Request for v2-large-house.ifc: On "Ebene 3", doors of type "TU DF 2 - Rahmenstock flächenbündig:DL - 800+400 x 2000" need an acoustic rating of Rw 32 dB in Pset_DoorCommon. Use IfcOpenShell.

First a look at what the model holds.

```python
import ifcopenshell
import ifcopenshell.util.element

model = ifcopenshell.open("v2-large-house.ifc")
print(model.schema)
storey = next(s for s in model.by_type("IfcBuildingStorey") if s.Name == "Ebene 3")
doors = [e for e in ifcopenshell.util.element.get_decomposition(storey) if e.is_a("IfcDoor")]
seen = {}
for e in doors:
    element_type = ifcopenshell.util.element.get_type(e)
    key = (element_type.Name if element_type != e and element_type else None, ifcopenshell.util.element.get_pset(e, "Pset_DoorCommon", "AcousticRating"))
    seen[key] = seen.get(key, 0) + 1
for (name, value), count in sorted(seen.items(), key=str):
    print(count, "x", name, "|", value)
```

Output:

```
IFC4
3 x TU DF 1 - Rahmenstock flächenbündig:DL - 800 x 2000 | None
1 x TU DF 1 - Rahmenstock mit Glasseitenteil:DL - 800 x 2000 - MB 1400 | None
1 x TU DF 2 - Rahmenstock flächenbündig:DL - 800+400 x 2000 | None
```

```python
import ifcopenshell
import ifcopenshell.api.pset
import ifcopenshell.util.element

model = ifcopenshell.open("v2-large-house.ifc")

storey = next(s for s in model.by_type("IfcBuildingStorey") if s.Name == "Ebene 3")
doors = [e for e in ifcopenshell.util.element.get_decomposition(storey) if e.is_a("IfcDoor")]

count = 0
for e in doors:
    element_type = ifcopenshell.util.element.get_type(e)
    if element_type in (None, e) or element_type.Name != "TU DF 2 - Rahmenstock flächenbündig:DL - 800+400 x 2000":
        continue
    # add_pset returns the element's existing set when there is one.
    pset = ifcopenshell.api.pset.add_pset(model, product=e, name="Pset_DoorCommon")
    ifcopenshell.api.pset.edit_pset(model, pset=pset, properties={"AcousticRating": "Rw 32 dB"})
    count += 1

print(count, "doors updated")

model.write("v2-large-house_updated.ifc")
```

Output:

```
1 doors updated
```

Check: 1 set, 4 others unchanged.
